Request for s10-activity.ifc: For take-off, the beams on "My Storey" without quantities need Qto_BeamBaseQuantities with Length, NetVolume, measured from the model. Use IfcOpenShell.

First a look at what the model holds.

```python
import ifcopenshell
import ifcopenshell.util.element
import ifcopenshell.util.unit

model = ifcopenshell.open("s10-activity.ifc")
print(model.schema)
for unit_type in ("LENGTHUNIT", "AREAUNIT", "VOLUMEUNIT"):
    print(unit_type, ifcopenshell.util.unit.calculate_unit_scale(model, unit_type))
storey = next(s for s in model.by_type("IfcBuildingStorey") if s.Name == "My Storey")
beams = [e for e in ifcopenshell.util.element.get_decomposition(storey) if e.is_a("IfcBeam")]
for e in sorted(beams, key=lambda e: e.id()):
    print(e.id(), e.is_a(), e.Name, list(ifcopenshell.util.element.get_psets(e, qtos_only=True)), sep=" | ")
```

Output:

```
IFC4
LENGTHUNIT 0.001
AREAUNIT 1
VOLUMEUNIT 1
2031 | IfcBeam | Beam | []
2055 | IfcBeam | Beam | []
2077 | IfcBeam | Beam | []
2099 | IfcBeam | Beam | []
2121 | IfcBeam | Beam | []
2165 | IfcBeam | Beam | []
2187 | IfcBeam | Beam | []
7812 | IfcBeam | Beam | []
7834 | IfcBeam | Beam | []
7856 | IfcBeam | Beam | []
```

```python
import ifcopenshell
import ifcopenshell.api.pset
import ifcopenshell.geom
import ifcopenshell.util.element
import ifcopenshell.util.shape
import ifcopenshell.util.unit

model = ifcopenshell.open("s10-activity.ifc")
unit_scale = ifcopenshell.util.unit.calculate_unit_scale(model)
volume_scale = ifcopenshell.util.unit.calculate_unit_scale(model, "VOLUMEUNIT")
settings = ifcopenshell.geom.settings()

storey = next(s for s in model.by_type("IfcBuildingStorey") if s.Name == "My Storey")
beams = [e for e in ifcopenshell.util.element.get_decomposition(storey) if e.is_a("IfcBeam")]

for e in sorted(beams, key=lambda e: e.id()):
    if ifcopenshell.util.element.get_psets(e, qtos_only=True, should_inherit=False):
        continue
    # Geometry comes back in metres, in the element's own axes.
    shape = ifcopenshell.geom.create_shape(settings, e)
    values = {
        "Length": ifcopenshell.util.shape.get_max_xyz(shape.geometry) / unit_scale,
        "NetVolume": ifcopenshell.util.shape.get_volume(shape.geometry) / volume_scale,
    }
    qto = ifcopenshell.api.pset.add_qto(model, product=e, name="Qto_BeamBaseQuantities")
    ifcopenshell.api.pset.edit_qto(model, qto=qto, properties=values)
    print(e.id(), {k: round(v, 3) for k, v in values.items()})

model.write("s10-activity_v2.ifc")
```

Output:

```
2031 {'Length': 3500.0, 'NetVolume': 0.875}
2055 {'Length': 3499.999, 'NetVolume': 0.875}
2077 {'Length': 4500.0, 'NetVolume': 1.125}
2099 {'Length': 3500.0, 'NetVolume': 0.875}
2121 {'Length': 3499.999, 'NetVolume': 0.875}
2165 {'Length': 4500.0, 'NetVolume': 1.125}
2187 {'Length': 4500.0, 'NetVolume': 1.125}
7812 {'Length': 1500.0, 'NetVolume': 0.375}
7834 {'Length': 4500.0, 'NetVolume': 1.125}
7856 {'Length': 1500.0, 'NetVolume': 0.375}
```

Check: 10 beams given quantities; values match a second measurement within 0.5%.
